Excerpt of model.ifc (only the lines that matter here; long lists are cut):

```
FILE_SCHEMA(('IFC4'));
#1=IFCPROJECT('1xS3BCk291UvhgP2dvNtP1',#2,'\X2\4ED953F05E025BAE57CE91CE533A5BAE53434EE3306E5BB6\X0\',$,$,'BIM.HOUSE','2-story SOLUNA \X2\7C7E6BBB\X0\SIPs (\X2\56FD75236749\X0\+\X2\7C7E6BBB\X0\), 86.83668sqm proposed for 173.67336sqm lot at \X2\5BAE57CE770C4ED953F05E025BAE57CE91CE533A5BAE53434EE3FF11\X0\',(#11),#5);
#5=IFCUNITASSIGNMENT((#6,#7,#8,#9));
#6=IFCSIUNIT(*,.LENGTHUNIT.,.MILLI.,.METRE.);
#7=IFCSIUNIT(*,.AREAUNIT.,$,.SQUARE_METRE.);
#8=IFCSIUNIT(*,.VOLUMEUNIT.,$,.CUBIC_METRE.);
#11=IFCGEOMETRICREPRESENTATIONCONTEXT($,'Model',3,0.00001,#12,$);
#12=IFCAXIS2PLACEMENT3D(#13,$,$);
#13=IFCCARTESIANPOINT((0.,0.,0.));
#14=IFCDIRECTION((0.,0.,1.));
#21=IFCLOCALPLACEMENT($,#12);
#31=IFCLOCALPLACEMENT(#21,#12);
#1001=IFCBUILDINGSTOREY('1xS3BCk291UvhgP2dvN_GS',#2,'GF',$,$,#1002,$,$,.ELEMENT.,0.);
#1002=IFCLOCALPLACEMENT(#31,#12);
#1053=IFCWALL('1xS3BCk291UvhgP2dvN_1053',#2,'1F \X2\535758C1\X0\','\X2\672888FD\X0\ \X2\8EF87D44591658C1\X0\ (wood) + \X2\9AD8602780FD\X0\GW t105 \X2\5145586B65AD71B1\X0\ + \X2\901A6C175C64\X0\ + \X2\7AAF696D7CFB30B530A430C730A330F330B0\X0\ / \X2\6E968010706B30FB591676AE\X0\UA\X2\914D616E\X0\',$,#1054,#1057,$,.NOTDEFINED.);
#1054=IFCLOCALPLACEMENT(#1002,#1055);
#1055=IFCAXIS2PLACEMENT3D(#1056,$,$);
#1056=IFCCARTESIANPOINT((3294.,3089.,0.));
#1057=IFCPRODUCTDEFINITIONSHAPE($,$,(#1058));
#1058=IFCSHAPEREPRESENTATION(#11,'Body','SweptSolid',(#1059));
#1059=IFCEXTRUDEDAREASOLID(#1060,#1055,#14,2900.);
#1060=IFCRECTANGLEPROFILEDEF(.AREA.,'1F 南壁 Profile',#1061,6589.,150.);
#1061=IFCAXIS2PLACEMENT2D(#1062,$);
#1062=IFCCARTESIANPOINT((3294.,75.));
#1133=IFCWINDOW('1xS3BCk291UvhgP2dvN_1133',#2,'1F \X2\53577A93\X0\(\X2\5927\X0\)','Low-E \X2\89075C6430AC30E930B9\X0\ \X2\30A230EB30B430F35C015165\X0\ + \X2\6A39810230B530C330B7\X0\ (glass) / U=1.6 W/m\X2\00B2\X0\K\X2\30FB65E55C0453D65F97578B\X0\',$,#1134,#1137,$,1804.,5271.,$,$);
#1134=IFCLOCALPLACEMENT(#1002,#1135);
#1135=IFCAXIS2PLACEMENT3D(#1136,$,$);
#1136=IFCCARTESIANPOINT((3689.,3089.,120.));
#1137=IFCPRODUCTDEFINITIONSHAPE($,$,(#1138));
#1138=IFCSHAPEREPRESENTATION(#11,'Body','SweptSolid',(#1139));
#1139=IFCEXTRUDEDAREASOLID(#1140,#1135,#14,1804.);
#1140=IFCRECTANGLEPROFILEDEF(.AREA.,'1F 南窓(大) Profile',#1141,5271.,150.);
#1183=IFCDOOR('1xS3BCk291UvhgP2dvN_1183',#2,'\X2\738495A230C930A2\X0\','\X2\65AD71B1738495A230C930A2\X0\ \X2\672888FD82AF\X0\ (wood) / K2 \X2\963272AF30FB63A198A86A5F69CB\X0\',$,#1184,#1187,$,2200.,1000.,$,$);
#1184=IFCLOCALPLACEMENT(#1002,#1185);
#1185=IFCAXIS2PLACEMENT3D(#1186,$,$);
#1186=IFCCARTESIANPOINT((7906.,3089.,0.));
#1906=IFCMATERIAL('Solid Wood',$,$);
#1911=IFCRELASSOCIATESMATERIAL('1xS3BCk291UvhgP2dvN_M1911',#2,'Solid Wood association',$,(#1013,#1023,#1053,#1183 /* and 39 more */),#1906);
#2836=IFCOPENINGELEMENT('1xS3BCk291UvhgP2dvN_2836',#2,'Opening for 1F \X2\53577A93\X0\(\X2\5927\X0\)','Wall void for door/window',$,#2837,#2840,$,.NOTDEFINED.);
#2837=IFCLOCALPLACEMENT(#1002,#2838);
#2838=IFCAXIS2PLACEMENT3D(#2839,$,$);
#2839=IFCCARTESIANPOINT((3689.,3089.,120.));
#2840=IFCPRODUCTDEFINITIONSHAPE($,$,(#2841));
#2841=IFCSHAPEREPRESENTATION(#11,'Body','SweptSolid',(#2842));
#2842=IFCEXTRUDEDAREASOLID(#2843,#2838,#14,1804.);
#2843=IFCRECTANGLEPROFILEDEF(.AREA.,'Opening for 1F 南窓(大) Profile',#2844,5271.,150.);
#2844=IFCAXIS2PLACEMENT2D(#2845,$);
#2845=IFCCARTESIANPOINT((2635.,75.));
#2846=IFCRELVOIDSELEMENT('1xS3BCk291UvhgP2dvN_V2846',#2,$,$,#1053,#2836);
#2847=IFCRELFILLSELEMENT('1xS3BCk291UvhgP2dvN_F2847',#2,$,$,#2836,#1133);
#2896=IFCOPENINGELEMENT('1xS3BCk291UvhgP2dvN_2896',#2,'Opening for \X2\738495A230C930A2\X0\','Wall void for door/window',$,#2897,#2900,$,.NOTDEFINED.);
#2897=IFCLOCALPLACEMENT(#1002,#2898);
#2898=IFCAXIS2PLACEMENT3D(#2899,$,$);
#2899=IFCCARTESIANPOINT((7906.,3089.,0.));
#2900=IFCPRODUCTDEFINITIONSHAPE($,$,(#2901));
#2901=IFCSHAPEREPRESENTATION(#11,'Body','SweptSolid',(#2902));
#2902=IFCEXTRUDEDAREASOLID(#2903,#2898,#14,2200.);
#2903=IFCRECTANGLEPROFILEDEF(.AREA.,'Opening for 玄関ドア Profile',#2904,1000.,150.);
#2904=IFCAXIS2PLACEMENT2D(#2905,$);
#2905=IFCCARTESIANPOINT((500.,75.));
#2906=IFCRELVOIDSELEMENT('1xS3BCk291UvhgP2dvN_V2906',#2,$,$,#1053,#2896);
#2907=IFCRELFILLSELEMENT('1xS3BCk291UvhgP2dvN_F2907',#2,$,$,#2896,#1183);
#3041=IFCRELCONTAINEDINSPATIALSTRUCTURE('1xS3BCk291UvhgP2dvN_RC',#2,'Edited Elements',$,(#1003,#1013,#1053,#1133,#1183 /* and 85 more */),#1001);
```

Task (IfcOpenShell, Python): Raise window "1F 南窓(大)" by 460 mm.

```python
import numpy as np
import ifcopenshell
import ifcopenshell.api.geometry
import ifcopenshell.util.placement
import ifcopenshell.util.unit

model = ifcopenshell.open("model.ifc")
unit_scale = ifcopenshell.util.unit.calculate_unit_scale(model)

window = model.by_guid("1xS3BCk291UvhgP2dvN_1133")
opening = window.FillsVoids[0].RelatingOpeningElement
dz = 460.0

shift = np.array([0.0, 0.0, dz])
# The window is not placed relative to its opening, so move both.
for product in (opening, window):
    matrix = ifcopenshell.util.placement.get_local_placement(product.ObjectPlacement)
    matrix[:3, 3] += shift
    ifcopenshell.api.geometry.edit_object_placement(model, product=product, matrix=matrix, is_si=False)

print(f"moved by {dz * unit_scale:+.3f} m")

model.write("model-out.ifc")
```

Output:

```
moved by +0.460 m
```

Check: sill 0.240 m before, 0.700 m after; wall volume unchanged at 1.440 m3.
